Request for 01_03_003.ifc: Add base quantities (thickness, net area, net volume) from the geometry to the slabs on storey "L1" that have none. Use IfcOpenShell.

First a look at what the model holds.

```python
import ifcopenshell
import ifcopenshell.util.element
import ifcopenshell.util.unit

model = ifcopenshell.open("01_03_003.ifc")
print(model.schema)
for unit_type in ("LENGTHUNIT", "AREAUNIT", "VOLUMEUNIT"):
    print(unit_type, ifcopenshell.util.unit.calculate_unit_scale(model, unit_type))
storey = next(s for s in model.by_type("IfcBuildingStorey") if s.Name == "L1")
slabs = [e for e in ifcopenshell.util.element.get_decomposition(storey) if e.is_a("IfcSlab")]
for e in sorted(slabs, key=lambda e: e.id()):
    print(e.id(), e.is_a(), e.Name, list(ifcopenshell.util.element.get_psets(e, qtos_only=True)), sep=" | ")
```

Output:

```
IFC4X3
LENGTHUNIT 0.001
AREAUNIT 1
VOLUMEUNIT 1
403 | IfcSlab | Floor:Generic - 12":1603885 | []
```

```python
import ifcopenshell
import ifcopenshell.api.pset
import ifcopenshell.geom
import ifcopenshell.util.element
import ifcopenshell.util.shape
import ifcopenshell.util.unit

model = ifcopenshell.open("01_03_003.ifc")
unit_scale = ifcopenshell.util.unit.calculate_unit_scale(model)
area_scale = ifcopenshell.util.unit.calculate_unit_scale(model, "AREAUNIT")
volume_scale = ifcopenshell.util.unit.calculate_unit_scale(model, "VOLUMEUNIT")
settings = ifcopenshell.geom.settings()

storey = next(s for s in model.by_type("IfcBuildingStorey") if s.Name == "L1")
slabs = [e for e in ifcopenshell.util.element.get_decomposition(storey) if e.is_a("IfcSlab")]

for e in sorted(slabs, key=lambda e: e.id()):
    if ifcopenshell.util.element.get_psets(e, qtos_only=True, should_inherit=False):
        continue
    # Geometry comes back in metres, in the element's own axes.
    shape = ifcopenshell.geom.create_shape(settings, e)
    values = {
        "Width": ifcopenshell.util.shape.get_z(shape.geometry) / unit_scale,
        "NetArea": ifcopenshell.util.shape.get_footprint_area(shape.geometry) / area_scale,
        "NetVolume": ifcopenshell.util.shape.get_volume(shape.geometry) / volume_scale,
    }
    qto = ifcopenshell.api.pset.add_qto(model, product=e, name="Qto_SlabBaseQuantities")
    ifcopenshell.api.pset.edit_qto(model, qto=qto, properties=values)
    print(e.id(), {k: round(v, 3) for k, v in values.items()})

model.write("01_03_003_edited.ifc")
```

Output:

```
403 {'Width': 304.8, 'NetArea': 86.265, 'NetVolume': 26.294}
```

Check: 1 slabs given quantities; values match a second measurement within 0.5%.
